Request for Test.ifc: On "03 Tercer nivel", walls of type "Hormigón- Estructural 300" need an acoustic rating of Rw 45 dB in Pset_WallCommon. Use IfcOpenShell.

First a look at what the model holds.

```python
import ifcopenshell
import ifcopenshell.util.element

model = ifcopenshell.open("Test.ifc")
print(model.schema)
storey = next(s for s in model.by_type("IfcBuildingStorey") if s.Name == "03 Tercer nivel")
walls = [e for e in ifcopenshell.util.element.get_decomposition(storey) if e.is_a("IfcWall")]
seen = {}
for e in walls:
    element_type = ifcopenshell.util.element.get_type(e)
    key = (element_type.Name if element_type != e and element_type else None, ifcopenshell.util.element.get_pset(e, "Pset_WallCommon", "AcousticRating"))
    seen[key] = seen.get(key, 0) + 1
for (name, value), count in sorted(seen.items(), key=str):
    print(count, "x", name, "|", value)
```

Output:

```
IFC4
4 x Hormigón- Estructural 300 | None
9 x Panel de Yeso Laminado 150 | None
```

```python
import ifcopenshell
import ifcopenshell.api.pset
import ifcopenshell.util.element

model = ifcopenshell.open("Test.ifc")

storey = next(s for s in model.by_type("IfcBuildingStorey") if s.Name == "03 Tercer nivel")
walls = [e for e in ifcopenshell.util.element.get_decomposition(storey) if e.is_a("IfcWall")]

count = 0
for e in walls:
    element_type = ifcopenshell.util.element.get_type(e)
    if element_type in (None, e) or element_type.Name != "Hormigón- Estructural 300":
        continue
    # add_pset returns the element's existing set when there is one.
    pset = ifcopenshell.api.pset.add_pset(model, product=e, name="Pset_WallCommon")
    ifcopenshell.api.pset.edit_pset(model, pset=pset, properties={"AcousticRating": "Rw 45 dB"})
    count += 1

print(count, "walls updated")

model.write("Test_v2.ifc")
```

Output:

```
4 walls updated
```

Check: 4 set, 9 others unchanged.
